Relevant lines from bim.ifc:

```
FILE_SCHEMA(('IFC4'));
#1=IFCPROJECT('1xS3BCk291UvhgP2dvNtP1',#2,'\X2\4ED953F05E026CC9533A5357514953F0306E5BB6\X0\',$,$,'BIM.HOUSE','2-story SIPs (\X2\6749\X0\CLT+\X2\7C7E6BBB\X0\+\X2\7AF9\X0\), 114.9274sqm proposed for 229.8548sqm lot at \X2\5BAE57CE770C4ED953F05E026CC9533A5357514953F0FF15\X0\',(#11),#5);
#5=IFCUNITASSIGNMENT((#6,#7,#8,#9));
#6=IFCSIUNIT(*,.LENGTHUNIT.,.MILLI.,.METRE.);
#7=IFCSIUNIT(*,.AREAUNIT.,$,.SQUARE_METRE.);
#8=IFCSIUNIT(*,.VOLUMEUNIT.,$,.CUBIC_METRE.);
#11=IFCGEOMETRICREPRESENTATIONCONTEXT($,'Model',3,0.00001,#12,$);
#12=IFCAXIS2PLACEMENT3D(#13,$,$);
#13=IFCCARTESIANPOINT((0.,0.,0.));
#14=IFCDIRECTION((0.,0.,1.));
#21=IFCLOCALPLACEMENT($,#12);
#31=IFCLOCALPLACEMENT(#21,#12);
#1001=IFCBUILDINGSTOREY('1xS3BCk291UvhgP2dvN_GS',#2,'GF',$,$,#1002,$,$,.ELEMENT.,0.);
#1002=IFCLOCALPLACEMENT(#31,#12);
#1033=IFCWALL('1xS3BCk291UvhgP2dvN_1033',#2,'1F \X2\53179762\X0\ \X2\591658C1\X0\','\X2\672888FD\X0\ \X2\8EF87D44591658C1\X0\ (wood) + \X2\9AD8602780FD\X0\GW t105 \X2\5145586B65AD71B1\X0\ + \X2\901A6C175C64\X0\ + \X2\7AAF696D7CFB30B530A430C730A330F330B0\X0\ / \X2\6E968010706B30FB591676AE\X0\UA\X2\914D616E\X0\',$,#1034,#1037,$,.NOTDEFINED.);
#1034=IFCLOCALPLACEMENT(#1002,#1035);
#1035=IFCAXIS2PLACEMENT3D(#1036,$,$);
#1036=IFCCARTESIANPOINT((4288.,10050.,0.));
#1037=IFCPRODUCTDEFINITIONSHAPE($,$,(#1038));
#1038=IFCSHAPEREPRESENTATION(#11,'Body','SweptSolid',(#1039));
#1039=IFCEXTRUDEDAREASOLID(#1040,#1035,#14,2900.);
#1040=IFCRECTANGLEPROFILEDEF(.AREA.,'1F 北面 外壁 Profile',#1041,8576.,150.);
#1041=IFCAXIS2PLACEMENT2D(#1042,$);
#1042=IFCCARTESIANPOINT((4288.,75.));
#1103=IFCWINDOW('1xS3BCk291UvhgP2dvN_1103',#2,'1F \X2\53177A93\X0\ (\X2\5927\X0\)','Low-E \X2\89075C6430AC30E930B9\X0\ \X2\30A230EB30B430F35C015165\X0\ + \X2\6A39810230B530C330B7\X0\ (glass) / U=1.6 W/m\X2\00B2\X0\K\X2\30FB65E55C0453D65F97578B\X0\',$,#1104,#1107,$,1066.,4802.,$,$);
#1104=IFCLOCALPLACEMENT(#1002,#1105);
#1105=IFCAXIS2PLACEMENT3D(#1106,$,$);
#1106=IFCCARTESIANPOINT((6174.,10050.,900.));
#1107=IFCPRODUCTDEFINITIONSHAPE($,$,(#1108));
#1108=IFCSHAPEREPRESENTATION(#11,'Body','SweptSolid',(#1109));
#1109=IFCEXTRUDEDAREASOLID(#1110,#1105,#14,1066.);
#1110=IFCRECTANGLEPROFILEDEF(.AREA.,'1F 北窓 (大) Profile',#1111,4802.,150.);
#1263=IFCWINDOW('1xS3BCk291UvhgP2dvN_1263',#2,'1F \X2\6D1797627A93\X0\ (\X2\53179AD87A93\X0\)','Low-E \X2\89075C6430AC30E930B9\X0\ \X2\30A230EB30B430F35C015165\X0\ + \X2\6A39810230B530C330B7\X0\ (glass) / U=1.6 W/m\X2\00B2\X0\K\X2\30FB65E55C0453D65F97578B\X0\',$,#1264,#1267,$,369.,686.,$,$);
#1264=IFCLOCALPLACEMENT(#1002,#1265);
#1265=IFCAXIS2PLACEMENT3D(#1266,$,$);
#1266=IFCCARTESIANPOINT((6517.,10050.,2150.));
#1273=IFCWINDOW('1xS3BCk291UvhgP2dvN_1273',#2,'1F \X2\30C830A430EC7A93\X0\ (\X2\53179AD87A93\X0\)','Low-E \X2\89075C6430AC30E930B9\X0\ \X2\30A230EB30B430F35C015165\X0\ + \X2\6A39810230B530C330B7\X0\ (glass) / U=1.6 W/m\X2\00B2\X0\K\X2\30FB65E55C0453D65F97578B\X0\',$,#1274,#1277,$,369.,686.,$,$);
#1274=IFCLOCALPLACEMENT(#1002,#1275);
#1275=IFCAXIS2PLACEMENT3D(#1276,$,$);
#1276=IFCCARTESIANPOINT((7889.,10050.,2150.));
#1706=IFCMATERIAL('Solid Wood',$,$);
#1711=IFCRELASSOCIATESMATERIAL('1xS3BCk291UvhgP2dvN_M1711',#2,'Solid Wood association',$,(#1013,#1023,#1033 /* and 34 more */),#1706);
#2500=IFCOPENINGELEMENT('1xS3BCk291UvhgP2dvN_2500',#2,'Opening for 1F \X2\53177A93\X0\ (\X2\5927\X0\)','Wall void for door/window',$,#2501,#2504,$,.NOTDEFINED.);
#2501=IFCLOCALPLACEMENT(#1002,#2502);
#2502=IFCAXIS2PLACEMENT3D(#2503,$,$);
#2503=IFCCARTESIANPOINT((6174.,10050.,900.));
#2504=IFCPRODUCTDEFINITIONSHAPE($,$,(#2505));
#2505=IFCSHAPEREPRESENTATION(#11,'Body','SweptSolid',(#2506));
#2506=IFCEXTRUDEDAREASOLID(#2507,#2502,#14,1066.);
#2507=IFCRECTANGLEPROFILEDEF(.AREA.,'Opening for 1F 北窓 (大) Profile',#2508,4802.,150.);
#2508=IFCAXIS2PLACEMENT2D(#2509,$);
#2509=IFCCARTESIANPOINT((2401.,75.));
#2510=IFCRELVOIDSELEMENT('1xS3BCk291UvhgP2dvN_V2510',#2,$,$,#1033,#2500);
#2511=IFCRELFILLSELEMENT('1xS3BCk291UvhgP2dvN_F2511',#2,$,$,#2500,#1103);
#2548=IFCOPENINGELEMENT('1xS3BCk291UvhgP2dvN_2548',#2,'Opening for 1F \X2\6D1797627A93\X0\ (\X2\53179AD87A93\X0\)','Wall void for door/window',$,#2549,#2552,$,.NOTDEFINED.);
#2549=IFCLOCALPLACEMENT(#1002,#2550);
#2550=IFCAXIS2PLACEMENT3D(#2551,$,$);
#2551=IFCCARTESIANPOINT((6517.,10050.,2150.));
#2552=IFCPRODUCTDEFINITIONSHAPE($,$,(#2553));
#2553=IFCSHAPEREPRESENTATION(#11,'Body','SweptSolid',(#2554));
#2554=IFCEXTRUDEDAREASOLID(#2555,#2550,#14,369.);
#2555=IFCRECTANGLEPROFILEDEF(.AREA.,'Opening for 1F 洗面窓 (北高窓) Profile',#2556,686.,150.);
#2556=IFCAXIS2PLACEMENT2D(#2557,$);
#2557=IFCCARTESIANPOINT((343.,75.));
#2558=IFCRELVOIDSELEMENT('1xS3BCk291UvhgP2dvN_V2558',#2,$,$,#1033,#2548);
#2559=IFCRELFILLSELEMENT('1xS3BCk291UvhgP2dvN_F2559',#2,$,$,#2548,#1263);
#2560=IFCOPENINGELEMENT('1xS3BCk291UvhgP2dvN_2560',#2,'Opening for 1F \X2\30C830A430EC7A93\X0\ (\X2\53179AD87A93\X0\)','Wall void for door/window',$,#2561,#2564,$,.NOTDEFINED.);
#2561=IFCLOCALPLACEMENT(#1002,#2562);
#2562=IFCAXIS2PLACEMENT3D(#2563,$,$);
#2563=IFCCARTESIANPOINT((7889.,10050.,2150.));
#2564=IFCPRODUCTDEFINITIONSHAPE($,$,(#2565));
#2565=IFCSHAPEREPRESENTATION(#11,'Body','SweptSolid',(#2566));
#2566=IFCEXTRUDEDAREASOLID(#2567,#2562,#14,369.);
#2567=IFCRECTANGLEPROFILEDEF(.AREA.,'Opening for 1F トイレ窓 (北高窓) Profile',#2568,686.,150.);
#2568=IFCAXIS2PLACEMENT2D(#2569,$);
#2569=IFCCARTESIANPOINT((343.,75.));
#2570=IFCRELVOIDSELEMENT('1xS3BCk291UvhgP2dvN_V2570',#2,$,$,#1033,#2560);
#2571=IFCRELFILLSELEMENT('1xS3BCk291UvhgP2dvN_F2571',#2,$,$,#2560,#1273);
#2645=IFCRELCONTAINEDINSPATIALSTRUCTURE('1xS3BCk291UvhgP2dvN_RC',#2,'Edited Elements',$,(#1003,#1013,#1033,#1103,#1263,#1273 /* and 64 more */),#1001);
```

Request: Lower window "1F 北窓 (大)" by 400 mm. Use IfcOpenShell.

```python
import numpy as np
import ifcopenshell
import ifcopenshell.api.geometry
import ifcopenshell.util.placement
import ifcopenshell.util.unit

model = ifcopenshell.open("bim.ifc")
unit_scale = ifcopenshell.util.unit.calculate_unit_scale(model)

window = model.by_guid("1xS3BCk291UvhgP2dvN_1103")
opening = window.FillsVoids[0].RelatingOpeningElement
dz = -0.4 / unit_scale

shift = np.array([0.0, 0.0, dz])
# The window is not placed relative to its opening, so move both.
for product in (opening, window):
    matrix = ifcopenshell.util.placement.get_local_placement(product.ObjectPlacement)
    matrix[:3, 3] += shift
    ifcopenshell.api.geometry.edit_object_placement(model, product=product, matrix=matrix, is_si=False)

print(f"moved by {dz * unit_scale:+.3f} m")

model.write("bim_edited.ifc")
```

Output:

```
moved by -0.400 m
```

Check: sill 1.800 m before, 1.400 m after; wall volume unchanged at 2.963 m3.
